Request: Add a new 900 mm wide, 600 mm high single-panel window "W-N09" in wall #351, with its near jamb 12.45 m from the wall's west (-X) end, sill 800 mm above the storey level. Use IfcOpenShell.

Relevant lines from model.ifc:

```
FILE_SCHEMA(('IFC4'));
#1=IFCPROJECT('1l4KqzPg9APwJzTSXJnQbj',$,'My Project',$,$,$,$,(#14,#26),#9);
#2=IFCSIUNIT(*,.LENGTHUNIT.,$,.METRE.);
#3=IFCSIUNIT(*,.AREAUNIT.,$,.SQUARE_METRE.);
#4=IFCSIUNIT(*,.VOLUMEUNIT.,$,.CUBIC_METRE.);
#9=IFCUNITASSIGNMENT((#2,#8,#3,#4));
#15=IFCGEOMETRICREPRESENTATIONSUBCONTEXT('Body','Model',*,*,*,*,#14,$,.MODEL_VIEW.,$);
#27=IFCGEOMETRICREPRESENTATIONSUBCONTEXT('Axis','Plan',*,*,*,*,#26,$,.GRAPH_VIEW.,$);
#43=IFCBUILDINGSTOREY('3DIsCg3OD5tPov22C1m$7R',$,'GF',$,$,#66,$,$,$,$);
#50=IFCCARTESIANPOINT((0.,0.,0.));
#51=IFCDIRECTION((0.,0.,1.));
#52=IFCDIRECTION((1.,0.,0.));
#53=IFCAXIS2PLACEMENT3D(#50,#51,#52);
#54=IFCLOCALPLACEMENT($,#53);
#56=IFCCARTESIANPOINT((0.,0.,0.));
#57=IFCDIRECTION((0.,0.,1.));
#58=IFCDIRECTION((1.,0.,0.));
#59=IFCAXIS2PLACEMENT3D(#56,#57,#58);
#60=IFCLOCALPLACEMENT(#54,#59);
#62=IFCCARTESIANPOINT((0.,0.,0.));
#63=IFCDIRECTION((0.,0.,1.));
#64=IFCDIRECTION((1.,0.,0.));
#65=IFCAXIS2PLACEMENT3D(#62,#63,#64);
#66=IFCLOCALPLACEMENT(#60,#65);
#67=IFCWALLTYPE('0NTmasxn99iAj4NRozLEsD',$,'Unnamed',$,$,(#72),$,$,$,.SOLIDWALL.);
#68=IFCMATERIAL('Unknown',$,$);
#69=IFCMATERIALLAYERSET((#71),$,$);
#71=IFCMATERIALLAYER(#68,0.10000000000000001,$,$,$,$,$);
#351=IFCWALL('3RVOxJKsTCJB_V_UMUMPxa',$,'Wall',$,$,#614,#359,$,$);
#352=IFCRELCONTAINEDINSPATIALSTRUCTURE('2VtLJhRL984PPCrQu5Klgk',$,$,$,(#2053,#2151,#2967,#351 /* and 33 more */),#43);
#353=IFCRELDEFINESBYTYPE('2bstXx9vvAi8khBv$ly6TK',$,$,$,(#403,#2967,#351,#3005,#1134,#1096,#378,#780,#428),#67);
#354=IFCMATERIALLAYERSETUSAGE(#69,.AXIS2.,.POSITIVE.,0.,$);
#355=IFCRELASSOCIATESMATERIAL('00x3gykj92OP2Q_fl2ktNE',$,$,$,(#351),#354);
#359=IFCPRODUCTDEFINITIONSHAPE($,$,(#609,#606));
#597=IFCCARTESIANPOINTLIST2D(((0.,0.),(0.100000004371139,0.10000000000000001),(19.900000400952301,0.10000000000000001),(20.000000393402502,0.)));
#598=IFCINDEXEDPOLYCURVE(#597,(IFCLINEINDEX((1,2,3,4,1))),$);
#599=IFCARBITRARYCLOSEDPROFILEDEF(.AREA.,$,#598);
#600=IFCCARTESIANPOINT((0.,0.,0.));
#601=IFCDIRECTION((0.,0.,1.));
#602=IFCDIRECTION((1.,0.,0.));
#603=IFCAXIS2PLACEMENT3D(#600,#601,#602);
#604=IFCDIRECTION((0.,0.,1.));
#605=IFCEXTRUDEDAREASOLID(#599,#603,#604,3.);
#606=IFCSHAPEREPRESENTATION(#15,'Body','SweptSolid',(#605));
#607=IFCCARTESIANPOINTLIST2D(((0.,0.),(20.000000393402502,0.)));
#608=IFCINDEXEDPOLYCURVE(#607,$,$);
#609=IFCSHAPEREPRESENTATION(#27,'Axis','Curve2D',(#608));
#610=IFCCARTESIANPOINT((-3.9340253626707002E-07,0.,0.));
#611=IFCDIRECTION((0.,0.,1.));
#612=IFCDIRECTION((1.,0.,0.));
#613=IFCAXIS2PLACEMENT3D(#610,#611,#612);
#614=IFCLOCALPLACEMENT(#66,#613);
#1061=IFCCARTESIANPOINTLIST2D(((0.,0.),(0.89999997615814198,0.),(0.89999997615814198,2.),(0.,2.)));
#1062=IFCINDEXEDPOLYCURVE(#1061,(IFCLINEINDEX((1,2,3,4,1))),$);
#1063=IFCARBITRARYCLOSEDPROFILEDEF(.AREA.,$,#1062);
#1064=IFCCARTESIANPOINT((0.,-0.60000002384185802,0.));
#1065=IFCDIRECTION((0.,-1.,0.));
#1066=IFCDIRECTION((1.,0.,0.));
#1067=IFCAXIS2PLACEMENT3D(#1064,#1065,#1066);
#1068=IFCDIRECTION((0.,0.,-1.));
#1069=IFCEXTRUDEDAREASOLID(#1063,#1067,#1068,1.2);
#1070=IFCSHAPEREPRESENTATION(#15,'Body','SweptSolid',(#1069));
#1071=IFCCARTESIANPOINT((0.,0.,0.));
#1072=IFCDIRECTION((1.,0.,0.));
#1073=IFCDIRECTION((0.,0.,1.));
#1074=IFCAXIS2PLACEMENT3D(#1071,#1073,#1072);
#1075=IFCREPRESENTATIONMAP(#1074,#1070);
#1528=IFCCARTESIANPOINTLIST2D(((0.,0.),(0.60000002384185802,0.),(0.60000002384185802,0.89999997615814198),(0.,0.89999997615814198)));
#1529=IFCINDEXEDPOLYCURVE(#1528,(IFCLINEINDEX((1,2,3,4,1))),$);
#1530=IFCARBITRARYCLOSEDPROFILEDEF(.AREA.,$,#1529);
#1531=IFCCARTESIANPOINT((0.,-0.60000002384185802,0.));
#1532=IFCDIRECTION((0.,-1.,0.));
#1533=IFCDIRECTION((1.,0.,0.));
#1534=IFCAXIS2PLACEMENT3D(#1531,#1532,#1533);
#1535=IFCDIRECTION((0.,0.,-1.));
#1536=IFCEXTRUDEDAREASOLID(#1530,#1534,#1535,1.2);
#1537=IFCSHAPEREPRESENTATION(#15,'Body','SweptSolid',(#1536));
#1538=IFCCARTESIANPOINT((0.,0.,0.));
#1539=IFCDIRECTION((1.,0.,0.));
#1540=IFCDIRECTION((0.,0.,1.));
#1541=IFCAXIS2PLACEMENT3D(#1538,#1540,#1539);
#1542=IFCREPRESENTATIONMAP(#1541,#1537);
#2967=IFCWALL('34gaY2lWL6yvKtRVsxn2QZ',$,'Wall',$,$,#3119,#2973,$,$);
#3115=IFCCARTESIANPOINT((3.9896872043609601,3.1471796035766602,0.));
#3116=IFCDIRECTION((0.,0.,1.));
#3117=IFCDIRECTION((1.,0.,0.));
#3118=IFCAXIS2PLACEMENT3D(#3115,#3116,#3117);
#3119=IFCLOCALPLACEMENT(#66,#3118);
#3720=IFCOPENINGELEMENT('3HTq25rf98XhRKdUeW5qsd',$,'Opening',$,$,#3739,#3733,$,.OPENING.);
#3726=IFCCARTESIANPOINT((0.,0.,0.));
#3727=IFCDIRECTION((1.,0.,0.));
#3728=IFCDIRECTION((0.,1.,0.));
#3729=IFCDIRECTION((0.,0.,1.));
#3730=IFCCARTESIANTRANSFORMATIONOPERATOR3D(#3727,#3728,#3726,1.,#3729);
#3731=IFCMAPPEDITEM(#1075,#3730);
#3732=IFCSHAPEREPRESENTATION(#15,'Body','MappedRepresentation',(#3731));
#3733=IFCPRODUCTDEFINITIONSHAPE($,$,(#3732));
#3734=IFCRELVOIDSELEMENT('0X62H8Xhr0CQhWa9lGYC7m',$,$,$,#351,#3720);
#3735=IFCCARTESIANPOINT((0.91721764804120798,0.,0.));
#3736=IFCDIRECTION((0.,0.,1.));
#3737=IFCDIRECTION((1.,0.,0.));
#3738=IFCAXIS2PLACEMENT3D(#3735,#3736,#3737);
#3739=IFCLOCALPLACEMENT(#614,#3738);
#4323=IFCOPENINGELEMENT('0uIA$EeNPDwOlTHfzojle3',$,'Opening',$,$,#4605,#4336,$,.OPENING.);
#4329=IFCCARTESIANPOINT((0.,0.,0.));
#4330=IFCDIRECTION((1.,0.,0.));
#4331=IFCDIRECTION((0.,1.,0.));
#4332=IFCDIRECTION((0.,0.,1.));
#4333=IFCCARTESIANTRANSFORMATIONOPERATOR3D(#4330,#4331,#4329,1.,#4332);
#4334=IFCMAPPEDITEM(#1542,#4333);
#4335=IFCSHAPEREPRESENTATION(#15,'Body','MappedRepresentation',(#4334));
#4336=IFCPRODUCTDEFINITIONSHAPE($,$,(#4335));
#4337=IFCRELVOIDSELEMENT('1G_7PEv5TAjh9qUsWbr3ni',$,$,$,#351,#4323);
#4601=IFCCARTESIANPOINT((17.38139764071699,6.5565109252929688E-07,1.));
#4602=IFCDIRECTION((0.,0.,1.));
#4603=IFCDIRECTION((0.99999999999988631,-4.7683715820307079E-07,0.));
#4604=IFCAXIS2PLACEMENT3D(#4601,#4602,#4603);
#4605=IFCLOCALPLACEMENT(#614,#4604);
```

```python
import numpy as np
import ifcopenshell
import ifcopenshell.api.feature
import ifcopenshell.api.geometry
import ifcopenshell.api.root
import ifcopenshell.api.spatial
import ifcopenshell.geom
import ifcopenshell.util.element
import ifcopenshell.util.placement
import ifcopenshell.util.representation
import ifcopenshell.util.shape
import ifcopenshell.util.unit

model = ifcopenshell.open("model.ifc")
unit_scale = ifcopenshell.util.unit.calculate_unit_scale(model)
settings = ifcopenshell.geom.settings()


def volume(element):
    """Net volume in cubic metres, openings subtracted."""
    shape = ifcopenshell.geom.create_shape(settings, element)
    return ifcopenshell.util.shape.get_volume(shape.geometry)


wall = model.by_guid("3RVOxJKsTCJB_V_UMUMPxa")
storey = ifcopenshell.util.element.get_container(wall, ifc_class="IfcBuildingStorey")
context = ifcopenshell.util.representation.get_context(model, "Model", "Body", "MODEL_VIEW")
before = volume(wall)

width, height, from_end, sill = 0.9, 0.6, 12.45, 0.8  # metres

# The wall runs along its own X axis, and the end named is its -X end.
wall_shape = ifcopenshell.geom.create_shape(settings, wall)
x, y, z = ifcopenshell.util.shape.get_vertices(wall_shape.geometry).T
start = x.min() + from_end
face, thickness = float(y.min()), float(y.max() - y.min())
wall_matrix = ifcopenshell.util.placement.get_local_placement(wall.ObjectPlacement)
level = ifcopenshell.util.placement.get_local_placement(storey.ObjectPlacement)[2, 3]


def in_wall(x, y):
    """Placement at x, y metres in the wall's axes, at sill height."""
    matrix = wall_matrix.copy()
    matrix[:, 3] = wall_matrix @ np.array([x / unit_scale, y / unit_scale, 0.0, 1.0])
    matrix[2, 3] = level + sill / unit_scale
    return matrix


# Opening: a box that overshoots both wall faces by 50 mm.
opening = ifcopenshell.api.root.create_entity(model, ifc_class="IfcOpeningElement", predefined_type="OPENING")
box = ifcopenshell.api.geometry.add_wall_representation(
    model, context=context, length=width, height=height, thickness=thickness + 0.1
)
ifcopenshell.api.geometry.assign_representation(model, product=opening, representation=box)
ifcopenshell.api.geometry.edit_object_placement(model, product=opening, matrix=in_wall(start, face - 0.05), is_si=False)
ifcopenshell.api.feature.add_feature(model, feature=opening, element=wall)

window = ifcopenshell.api.root.create_entity(model, ifc_class="IfcWindow", name="W-N09", predefined_type="WINDOW")
window.OverallWidth, window.OverallHeight = width / unit_scale, height / unit_scale
window.PartitioningType = "SINGLE_PANEL"
body = ifcopenshell.api.geometry.add_window_representation(
    model,
    context=context,
    overall_width=window.OverallWidth,
    overall_height=window.OverallHeight,
    partition_type="SINGLE_PANEL",
)
ifcopenshell.api.geometry.assign_representation(model, product=window, representation=body)
ifcopenshell.api.spatial.assign_container(model, products=[window], relating_structure=storey)
ifcopenshell.api.feature.add_filling(model, opening=opening, element=window)

# Centre the window in the wall's thickness.
ifcopenshell.api.geometry.edit_object_placement(model, product=window, matrix=in_wall(start, face), is_si=False)
window_shape = ifcopenshell.geom.create_shape(settings, window)
depth = ifcopenshell.util.shape.get_vertices(window_shape.geometry)[:, 1]
offset = face + thickness / 2 - (depth.min() + depth.max()) / 2
ifcopenshell.api.geometry.edit_object_placement(model, product=window, matrix=in_wall(start, offset), is_si=False)

after = volume(wall)

print(f"wall volume {before:.3f} -> {after:.3f} m3")

model.write("model_edited.ifc")
```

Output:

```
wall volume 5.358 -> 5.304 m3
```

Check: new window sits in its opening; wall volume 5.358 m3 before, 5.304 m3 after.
